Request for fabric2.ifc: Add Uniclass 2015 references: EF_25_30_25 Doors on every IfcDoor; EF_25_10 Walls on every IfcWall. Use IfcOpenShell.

First a look at what the model holds.

```python
import ifcopenshell

model = ifcopenshell.open("fabric2.ifc")
print(model.schema)
print("classifications:", [c.Name for c in model.by_type("IfcClassification")])
for ifc_class in ("IfcDoor", "IfcRoof", "IfcStair", "IfcWall", "IfcWindow"):
    print(ifc_class, len(model.by_type(ifc_class)))
```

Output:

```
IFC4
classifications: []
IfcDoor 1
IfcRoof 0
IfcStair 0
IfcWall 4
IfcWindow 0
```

```python
import ifcopenshell
import ifcopenshell.api.classification

model = ifcopenshell.open("fabric2.ifc")

system = ifcopenshell.api.classification.add_classification(model, classification="Uniclass 2015")

codes = {
    "IfcDoor": ("EF_25_30_25", "Doors"),
    "IfcWall": ("EF_25_10", "Walls"),
}
for ifc_class, (code, name) in codes.items():
    products = model.by_type(ifc_class)
    ifcopenshell.api.classification.add_reference(
        model, products=products, classification=system, identification=code, name=name
    )
    print(code, len(products))

model.write("fabric2_updated.ifc")
```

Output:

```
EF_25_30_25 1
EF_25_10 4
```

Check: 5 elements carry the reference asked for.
